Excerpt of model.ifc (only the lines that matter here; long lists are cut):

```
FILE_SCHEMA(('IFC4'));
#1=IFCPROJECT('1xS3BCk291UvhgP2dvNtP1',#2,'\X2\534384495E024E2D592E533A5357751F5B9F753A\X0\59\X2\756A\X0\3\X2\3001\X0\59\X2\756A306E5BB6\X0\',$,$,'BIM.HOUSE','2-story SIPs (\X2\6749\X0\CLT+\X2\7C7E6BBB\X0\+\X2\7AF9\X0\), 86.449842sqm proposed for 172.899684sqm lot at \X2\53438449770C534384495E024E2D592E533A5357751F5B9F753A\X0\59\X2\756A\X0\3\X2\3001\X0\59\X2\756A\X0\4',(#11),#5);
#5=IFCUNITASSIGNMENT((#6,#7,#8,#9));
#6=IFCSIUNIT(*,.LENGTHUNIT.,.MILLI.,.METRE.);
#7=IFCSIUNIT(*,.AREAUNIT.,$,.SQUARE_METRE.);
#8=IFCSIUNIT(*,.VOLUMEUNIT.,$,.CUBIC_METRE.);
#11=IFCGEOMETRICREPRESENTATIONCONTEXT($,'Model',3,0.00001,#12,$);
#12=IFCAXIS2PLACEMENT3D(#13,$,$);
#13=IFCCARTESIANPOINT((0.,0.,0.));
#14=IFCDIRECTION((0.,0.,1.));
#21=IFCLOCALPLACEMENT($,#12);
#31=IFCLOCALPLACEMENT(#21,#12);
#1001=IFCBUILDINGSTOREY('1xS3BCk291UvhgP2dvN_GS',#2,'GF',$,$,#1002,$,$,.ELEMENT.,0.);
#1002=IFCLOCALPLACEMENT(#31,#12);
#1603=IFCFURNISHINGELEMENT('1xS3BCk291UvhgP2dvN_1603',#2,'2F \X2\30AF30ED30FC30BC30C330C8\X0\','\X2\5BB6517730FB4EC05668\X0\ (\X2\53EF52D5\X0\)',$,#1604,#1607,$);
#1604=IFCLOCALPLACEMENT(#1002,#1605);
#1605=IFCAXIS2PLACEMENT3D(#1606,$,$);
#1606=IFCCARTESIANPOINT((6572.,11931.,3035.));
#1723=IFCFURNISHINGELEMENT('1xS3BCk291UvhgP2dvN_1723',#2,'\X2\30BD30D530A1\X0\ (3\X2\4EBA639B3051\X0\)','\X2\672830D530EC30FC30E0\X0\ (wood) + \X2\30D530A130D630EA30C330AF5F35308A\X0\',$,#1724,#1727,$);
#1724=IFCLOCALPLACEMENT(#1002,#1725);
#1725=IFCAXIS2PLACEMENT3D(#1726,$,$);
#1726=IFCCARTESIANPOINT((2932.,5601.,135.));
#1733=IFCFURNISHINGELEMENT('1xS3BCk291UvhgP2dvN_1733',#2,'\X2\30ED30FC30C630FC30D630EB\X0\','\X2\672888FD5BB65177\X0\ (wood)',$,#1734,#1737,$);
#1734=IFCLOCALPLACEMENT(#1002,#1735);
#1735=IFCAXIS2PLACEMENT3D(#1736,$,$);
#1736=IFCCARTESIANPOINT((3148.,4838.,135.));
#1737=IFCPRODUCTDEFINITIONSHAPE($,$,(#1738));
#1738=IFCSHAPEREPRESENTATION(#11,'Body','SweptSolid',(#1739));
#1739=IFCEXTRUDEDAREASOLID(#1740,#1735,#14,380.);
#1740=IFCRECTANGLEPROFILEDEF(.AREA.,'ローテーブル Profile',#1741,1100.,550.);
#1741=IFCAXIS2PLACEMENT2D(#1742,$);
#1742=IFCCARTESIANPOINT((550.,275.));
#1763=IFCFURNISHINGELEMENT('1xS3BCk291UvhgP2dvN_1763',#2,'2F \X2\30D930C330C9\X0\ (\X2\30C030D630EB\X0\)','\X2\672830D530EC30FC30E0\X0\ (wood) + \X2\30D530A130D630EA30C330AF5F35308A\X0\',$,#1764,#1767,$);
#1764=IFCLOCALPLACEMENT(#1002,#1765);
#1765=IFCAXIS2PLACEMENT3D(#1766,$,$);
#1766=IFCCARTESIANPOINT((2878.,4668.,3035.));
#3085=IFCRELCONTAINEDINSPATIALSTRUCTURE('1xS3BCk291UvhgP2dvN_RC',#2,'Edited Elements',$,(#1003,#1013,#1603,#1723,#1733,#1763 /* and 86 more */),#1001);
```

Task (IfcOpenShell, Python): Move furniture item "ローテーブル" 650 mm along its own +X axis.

```python
import ifcopenshell
import ifcopenshell.api.geometry
import ifcopenshell.util.placement

model = ifcopenshell.open("model.ifc")

item = model.by_id(1733)
matrix = ifcopenshell.util.placement.get_local_placement(item.ObjectPlacement)
matrix[:3, 3] += matrix[:3, 0] * 650.0
ifcopenshell.api.geometry.edit_object_placement(model, product=item, matrix=matrix, is_si=False)

print(ifcopenshell.util.placement.get_local_placement(item.ObjectPlacement).round(3) + 0.0)

model.write("model_updated.ifc")
```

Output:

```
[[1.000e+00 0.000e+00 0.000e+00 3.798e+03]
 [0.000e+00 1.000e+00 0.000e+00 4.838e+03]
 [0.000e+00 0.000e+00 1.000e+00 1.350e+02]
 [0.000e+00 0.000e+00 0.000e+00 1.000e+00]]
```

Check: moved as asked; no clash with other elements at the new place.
